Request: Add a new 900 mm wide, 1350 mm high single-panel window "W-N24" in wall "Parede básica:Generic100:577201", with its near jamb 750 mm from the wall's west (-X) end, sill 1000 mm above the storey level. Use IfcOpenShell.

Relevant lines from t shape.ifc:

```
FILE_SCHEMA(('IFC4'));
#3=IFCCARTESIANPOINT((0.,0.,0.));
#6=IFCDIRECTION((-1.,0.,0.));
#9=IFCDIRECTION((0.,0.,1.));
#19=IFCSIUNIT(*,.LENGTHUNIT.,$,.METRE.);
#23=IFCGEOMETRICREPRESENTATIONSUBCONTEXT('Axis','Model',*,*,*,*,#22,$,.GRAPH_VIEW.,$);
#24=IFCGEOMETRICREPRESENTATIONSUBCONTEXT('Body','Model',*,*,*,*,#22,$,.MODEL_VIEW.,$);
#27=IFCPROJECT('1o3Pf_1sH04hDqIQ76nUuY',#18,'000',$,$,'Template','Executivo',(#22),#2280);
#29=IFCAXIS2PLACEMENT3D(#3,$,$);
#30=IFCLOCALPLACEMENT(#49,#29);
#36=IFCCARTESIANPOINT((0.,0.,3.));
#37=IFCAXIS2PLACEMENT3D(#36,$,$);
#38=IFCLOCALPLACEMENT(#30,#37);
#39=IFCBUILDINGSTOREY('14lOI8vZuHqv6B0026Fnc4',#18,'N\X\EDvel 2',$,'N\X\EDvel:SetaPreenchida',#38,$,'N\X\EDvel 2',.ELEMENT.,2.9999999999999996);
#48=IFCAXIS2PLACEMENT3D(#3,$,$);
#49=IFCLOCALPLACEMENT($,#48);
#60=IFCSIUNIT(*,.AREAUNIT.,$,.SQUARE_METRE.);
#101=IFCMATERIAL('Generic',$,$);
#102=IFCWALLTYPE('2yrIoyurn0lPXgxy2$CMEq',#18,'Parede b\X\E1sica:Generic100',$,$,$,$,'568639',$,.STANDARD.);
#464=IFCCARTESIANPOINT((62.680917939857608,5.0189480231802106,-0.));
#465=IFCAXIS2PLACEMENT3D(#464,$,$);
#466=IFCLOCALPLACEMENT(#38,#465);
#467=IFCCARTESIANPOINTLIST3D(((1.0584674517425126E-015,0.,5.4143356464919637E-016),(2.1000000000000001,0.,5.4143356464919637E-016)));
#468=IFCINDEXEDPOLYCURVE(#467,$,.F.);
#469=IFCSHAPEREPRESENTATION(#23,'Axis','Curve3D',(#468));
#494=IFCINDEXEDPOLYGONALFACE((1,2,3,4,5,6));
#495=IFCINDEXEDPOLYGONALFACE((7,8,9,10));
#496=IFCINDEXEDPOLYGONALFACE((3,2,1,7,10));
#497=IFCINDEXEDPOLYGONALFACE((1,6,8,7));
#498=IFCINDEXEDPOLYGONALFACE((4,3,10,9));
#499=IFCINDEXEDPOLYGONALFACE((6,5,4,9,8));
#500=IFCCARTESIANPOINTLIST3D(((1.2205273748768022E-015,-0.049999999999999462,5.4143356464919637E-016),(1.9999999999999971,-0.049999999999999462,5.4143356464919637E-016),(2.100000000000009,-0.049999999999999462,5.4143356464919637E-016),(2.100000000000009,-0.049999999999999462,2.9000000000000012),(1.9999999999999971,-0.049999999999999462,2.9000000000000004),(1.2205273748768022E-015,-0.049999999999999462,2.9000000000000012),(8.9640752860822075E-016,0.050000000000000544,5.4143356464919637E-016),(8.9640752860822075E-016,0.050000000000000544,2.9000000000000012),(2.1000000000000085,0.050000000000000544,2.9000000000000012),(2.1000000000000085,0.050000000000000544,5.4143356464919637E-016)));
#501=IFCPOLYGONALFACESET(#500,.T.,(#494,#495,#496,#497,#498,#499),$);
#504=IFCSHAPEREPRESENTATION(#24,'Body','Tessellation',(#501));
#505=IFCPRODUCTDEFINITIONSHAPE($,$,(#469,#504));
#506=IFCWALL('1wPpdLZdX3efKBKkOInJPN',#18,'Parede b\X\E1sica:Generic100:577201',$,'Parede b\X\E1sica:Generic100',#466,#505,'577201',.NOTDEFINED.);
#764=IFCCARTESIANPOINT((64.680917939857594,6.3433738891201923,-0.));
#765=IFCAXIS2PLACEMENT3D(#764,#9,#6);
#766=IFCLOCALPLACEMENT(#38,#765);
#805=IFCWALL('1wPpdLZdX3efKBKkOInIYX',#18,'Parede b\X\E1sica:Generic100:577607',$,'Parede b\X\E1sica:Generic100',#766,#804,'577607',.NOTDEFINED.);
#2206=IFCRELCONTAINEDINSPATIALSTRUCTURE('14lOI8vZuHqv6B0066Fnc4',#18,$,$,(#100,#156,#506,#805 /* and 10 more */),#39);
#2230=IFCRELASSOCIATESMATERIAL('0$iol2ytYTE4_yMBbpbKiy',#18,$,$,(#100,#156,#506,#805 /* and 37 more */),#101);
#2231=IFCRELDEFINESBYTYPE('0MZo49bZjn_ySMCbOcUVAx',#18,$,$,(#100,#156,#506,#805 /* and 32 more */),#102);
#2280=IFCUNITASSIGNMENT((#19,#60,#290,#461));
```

```python
import numpy as np
import ifcopenshell
import ifcopenshell.api.feature
import ifcopenshell.api.geometry
import ifcopenshell.api.root
import ifcopenshell.api.spatial
import ifcopenshell.geom
import ifcopenshell.util.element
import ifcopenshell.util.placement
import ifcopenshell.util.representation
import ifcopenshell.util.shape
import ifcopenshell.util.unit

model = ifcopenshell.open("t shape.ifc")
unit_scale = ifcopenshell.util.unit.calculate_unit_scale(model)
settings = ifcopenshell.geom.settings()


def volume(element):
    """Net volume in cubic metres, openings subtracted."""
    shape = ifcopenshell.geom.create_shape(settings, element)
    return ifcopenshell.util.shape.get_volume(shape.geometry)


wall = model.by_id(506)
storey = ifcopenshell.util.element.get_container(wall, ifc_class="IfcBuildingStorey")
context = ifcopenshell.util.representation.get_context(model, "Model", "Body", "MODEL_VIEW")
before = volume(wall)

width, height, from_end, sill = 0.9, 1.35, 0.75, 1  # metres

# The wall runs along its own X axis, and the end named is its -X end.
wall_shape = ifcopenshell.geom.create_shape(settings, wall)
x, y, z = ifcopenshell.util.shape.get_vertices(wall_shape.geometry).T
start = x.min() + from_end
face, thickness = float(y.min()), float(y.max() - y.min())
wall_matrix = ifcopenshell.util.placement.get_local_placement(wall.ObjectPlacement)
level = ifcopenshell.util.placement.get_local_placement(storey.ObjectPlacement)[2, 3]


def in_wall(x, y):
    """Placement at x, y metres in the wall's axes, at sill height."""
    matrix = wall_matrix.copy()
    matrix[:, 3] = wall_matrix @ np.array([x / unit_scale, y / unit_scale, 0.0, 1.0])
    matrix[2, 3] = level + sill / unit_scale
    return matrix


# Opening: a box that overshoots both wall faces by 50 mm.
opening = ifcopenshell.api.root.create_entity(model, ifc_class="IfcOpeningElement", predefined_type="OPENING")
box = ifcopenshell.api.geometry.add_wall_representation(
    model, context=context, length=width, height=height, thickness=thickness + 0.1
)
ifcopenshell.api.geometry.assign_representation(model, product=opening, representation=box)
ifcopenshell.api.geometry.edit_object_placement(model, product=opening, matrix=in_wall(start, face - 0.05), is_si=False)
ifcopenshell.api.feature.add_feature(model, feature=opening, element=wall)

window = ifcopenshell.api.root.create_entity(model, ifc_class="IfcWindow", name="W-N24", predefined_type="WINDOW")
window.OverallWidth, window.OverallHeight = width / unit_scale, height / unit_scale
window.PartitioningType = "SINGLE_PANEL"
body = ifcopenshell.api.geometry.add_window_representation(
    model,
    context=context,
    overall_width=window.OverallWidth,
    overall_height=window.OverallHeight,
    partition_type="SINGLE_PANEL",
)
ifcopenshell.api.geometry.assign_representation(model, product=window, representation=body)
ifcopenshell.api.spatial.assign_container(model, products=[window], relating_structure=storey)
ifcopenshell.api.feature.add_filling(model, opening=opening, element=window)

# Centre the window in the wall's thickness.
ifcopenshell.api.geometry.edit_object_placement(model, product=window, matrix=in_wall(start, face), is_si=False)
window_shape = ifcopenshell.geom.create_shape(settings, window)
depth = ifcopenshell.util.shape.get_vertices(window_shape.geometry)[:, 1]
offset = face + thickness / 2 - (depth.min() + depth.max()) / 2
ifcopenshell.api.geometry.edit_object_placement(model, product=window, matrix=in_wall(start, offset), is_si=False)

after = volume(wall)

print(f"wall volume {before:.3f} -> {after:.3f} m3")

model.write("t shape_edited.ifc")
```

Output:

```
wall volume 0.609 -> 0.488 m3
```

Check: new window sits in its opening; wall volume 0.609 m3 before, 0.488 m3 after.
